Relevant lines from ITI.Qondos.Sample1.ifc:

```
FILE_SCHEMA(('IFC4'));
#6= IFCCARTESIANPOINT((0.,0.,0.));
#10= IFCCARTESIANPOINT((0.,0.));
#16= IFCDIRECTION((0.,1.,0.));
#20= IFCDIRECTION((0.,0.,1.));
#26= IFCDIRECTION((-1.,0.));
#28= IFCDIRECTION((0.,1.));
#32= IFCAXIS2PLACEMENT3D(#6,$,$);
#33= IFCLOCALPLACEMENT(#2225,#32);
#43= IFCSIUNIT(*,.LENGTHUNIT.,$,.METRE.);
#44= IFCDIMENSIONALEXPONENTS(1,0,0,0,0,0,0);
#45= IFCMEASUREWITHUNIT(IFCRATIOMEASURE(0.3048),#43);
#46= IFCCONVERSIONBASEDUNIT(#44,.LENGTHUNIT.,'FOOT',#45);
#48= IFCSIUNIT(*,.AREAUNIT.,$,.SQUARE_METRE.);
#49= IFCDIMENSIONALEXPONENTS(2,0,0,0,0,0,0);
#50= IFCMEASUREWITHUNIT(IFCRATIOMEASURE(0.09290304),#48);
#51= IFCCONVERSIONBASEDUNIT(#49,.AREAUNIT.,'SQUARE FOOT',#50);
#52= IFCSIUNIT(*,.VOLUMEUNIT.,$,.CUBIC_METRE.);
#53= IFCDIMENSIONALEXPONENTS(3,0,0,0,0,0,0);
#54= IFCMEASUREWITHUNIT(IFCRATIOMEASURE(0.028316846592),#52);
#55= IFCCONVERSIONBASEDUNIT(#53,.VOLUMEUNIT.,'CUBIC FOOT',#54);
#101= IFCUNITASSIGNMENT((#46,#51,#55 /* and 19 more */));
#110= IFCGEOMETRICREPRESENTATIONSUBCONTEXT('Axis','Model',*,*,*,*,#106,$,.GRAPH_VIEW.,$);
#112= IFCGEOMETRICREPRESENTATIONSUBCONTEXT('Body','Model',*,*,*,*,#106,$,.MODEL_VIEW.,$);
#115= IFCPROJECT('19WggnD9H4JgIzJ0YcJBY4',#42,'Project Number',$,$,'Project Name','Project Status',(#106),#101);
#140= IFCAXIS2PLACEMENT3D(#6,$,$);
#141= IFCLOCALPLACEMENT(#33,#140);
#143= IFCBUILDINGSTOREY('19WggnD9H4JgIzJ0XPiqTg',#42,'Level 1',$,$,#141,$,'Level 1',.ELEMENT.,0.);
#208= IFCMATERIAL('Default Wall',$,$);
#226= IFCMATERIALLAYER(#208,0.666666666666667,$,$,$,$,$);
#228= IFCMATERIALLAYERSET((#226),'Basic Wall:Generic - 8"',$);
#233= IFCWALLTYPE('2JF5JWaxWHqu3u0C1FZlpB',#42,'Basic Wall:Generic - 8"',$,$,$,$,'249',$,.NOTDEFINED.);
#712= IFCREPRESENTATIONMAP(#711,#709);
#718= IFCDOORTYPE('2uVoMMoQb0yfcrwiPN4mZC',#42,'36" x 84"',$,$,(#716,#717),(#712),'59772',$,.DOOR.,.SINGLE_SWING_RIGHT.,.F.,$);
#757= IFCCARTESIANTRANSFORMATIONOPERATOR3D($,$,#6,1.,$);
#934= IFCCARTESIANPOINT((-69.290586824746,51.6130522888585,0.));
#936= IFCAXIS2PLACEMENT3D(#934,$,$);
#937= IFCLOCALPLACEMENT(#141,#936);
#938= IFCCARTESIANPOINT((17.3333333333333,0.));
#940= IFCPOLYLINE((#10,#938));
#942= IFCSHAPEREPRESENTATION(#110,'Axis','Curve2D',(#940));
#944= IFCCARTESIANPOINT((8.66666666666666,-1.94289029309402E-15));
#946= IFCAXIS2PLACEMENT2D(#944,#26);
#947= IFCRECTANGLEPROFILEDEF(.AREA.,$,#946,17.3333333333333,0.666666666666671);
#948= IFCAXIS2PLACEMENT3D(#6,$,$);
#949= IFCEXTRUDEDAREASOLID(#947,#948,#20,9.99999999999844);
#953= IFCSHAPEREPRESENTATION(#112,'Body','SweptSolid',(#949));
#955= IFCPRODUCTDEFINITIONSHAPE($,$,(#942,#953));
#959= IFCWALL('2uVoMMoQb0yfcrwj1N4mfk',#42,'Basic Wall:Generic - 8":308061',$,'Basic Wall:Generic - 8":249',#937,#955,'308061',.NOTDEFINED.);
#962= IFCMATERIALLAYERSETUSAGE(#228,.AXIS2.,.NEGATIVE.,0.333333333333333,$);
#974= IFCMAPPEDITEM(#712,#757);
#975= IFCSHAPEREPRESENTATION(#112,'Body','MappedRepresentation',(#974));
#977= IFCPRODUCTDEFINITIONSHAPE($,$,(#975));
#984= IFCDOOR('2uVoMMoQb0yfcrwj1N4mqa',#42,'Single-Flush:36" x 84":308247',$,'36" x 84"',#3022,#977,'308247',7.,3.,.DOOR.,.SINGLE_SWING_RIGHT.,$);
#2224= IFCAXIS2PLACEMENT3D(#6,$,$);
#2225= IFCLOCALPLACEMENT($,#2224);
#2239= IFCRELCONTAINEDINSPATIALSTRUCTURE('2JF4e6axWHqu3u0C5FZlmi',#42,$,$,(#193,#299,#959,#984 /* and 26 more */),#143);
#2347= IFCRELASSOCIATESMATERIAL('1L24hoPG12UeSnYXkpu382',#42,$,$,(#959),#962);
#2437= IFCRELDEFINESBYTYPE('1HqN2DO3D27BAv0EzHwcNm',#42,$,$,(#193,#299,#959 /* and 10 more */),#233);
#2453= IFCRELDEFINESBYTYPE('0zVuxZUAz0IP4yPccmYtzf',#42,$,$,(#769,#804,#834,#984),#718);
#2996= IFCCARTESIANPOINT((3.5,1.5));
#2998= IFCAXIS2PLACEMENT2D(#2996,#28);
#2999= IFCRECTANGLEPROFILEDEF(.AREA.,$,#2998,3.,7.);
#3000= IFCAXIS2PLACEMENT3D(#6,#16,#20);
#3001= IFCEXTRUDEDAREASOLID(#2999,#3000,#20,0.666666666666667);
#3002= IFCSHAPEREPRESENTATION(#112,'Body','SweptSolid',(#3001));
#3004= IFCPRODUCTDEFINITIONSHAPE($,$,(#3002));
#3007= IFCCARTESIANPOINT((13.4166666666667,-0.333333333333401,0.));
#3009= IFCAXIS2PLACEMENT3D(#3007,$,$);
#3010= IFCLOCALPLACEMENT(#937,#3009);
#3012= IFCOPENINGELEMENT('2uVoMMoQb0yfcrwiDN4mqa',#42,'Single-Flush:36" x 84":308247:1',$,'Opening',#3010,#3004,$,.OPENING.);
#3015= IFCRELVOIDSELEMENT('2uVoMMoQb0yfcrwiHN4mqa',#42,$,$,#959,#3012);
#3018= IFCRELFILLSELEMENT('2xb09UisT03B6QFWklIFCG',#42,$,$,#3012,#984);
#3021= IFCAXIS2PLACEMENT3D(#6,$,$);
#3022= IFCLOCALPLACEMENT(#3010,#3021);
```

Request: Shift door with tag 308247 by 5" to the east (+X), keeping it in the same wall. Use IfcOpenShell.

```python
import ifcopenshell
import ifcopenshell.api.geometry
import ifcopenshell.util.placement
import ifcopenshell.util.unit

model = ifcopenshell.open("ITI.Qondos.Sample1.ifc")
unit_scale = ifcopenshell.util.unit.calculate_unit_scale(model)

door = model.by_guid("2uVoMMoQb0yfcrwj1N4mqa")
opening = door.FillsVoids[0].RelatingOpeningElement
wall = opening.VoidsElements[0].RelatingBuildingElement

wall_matrix = ifcopenshell.util.placement.get_local_placement(wall.ObjectPlacement)
shift = wall_matrix[:3, 0] * 5 * 0.0254 / unit_scale
before = ifcopenshell.util.placement.get_local_placement(door.ObjectPlacement)[:3, 3].copy()

# The door is placed relative to its opening, so it follows when the opening moves.
matrix = ifcopenshell.util.placement.get_local_placement(opening.ObjectPlacement)
matrix[:3, 3] += shift
ifcopenshell.api.geometry.edit_object_placement(
    model, product=opening, matrix=matrix, is_si=False, should_transform_children=True
)

after = ifcopenshell.util.placement.get_local_placement(door.ObjectPlacement)[:3, 3]
print("door moved by", (after - before).round(3) + 0.0)

model.write("ITI.Qondos.Sample1-out.ifc")
```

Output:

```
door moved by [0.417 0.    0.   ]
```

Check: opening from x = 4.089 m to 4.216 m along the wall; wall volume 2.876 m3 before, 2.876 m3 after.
